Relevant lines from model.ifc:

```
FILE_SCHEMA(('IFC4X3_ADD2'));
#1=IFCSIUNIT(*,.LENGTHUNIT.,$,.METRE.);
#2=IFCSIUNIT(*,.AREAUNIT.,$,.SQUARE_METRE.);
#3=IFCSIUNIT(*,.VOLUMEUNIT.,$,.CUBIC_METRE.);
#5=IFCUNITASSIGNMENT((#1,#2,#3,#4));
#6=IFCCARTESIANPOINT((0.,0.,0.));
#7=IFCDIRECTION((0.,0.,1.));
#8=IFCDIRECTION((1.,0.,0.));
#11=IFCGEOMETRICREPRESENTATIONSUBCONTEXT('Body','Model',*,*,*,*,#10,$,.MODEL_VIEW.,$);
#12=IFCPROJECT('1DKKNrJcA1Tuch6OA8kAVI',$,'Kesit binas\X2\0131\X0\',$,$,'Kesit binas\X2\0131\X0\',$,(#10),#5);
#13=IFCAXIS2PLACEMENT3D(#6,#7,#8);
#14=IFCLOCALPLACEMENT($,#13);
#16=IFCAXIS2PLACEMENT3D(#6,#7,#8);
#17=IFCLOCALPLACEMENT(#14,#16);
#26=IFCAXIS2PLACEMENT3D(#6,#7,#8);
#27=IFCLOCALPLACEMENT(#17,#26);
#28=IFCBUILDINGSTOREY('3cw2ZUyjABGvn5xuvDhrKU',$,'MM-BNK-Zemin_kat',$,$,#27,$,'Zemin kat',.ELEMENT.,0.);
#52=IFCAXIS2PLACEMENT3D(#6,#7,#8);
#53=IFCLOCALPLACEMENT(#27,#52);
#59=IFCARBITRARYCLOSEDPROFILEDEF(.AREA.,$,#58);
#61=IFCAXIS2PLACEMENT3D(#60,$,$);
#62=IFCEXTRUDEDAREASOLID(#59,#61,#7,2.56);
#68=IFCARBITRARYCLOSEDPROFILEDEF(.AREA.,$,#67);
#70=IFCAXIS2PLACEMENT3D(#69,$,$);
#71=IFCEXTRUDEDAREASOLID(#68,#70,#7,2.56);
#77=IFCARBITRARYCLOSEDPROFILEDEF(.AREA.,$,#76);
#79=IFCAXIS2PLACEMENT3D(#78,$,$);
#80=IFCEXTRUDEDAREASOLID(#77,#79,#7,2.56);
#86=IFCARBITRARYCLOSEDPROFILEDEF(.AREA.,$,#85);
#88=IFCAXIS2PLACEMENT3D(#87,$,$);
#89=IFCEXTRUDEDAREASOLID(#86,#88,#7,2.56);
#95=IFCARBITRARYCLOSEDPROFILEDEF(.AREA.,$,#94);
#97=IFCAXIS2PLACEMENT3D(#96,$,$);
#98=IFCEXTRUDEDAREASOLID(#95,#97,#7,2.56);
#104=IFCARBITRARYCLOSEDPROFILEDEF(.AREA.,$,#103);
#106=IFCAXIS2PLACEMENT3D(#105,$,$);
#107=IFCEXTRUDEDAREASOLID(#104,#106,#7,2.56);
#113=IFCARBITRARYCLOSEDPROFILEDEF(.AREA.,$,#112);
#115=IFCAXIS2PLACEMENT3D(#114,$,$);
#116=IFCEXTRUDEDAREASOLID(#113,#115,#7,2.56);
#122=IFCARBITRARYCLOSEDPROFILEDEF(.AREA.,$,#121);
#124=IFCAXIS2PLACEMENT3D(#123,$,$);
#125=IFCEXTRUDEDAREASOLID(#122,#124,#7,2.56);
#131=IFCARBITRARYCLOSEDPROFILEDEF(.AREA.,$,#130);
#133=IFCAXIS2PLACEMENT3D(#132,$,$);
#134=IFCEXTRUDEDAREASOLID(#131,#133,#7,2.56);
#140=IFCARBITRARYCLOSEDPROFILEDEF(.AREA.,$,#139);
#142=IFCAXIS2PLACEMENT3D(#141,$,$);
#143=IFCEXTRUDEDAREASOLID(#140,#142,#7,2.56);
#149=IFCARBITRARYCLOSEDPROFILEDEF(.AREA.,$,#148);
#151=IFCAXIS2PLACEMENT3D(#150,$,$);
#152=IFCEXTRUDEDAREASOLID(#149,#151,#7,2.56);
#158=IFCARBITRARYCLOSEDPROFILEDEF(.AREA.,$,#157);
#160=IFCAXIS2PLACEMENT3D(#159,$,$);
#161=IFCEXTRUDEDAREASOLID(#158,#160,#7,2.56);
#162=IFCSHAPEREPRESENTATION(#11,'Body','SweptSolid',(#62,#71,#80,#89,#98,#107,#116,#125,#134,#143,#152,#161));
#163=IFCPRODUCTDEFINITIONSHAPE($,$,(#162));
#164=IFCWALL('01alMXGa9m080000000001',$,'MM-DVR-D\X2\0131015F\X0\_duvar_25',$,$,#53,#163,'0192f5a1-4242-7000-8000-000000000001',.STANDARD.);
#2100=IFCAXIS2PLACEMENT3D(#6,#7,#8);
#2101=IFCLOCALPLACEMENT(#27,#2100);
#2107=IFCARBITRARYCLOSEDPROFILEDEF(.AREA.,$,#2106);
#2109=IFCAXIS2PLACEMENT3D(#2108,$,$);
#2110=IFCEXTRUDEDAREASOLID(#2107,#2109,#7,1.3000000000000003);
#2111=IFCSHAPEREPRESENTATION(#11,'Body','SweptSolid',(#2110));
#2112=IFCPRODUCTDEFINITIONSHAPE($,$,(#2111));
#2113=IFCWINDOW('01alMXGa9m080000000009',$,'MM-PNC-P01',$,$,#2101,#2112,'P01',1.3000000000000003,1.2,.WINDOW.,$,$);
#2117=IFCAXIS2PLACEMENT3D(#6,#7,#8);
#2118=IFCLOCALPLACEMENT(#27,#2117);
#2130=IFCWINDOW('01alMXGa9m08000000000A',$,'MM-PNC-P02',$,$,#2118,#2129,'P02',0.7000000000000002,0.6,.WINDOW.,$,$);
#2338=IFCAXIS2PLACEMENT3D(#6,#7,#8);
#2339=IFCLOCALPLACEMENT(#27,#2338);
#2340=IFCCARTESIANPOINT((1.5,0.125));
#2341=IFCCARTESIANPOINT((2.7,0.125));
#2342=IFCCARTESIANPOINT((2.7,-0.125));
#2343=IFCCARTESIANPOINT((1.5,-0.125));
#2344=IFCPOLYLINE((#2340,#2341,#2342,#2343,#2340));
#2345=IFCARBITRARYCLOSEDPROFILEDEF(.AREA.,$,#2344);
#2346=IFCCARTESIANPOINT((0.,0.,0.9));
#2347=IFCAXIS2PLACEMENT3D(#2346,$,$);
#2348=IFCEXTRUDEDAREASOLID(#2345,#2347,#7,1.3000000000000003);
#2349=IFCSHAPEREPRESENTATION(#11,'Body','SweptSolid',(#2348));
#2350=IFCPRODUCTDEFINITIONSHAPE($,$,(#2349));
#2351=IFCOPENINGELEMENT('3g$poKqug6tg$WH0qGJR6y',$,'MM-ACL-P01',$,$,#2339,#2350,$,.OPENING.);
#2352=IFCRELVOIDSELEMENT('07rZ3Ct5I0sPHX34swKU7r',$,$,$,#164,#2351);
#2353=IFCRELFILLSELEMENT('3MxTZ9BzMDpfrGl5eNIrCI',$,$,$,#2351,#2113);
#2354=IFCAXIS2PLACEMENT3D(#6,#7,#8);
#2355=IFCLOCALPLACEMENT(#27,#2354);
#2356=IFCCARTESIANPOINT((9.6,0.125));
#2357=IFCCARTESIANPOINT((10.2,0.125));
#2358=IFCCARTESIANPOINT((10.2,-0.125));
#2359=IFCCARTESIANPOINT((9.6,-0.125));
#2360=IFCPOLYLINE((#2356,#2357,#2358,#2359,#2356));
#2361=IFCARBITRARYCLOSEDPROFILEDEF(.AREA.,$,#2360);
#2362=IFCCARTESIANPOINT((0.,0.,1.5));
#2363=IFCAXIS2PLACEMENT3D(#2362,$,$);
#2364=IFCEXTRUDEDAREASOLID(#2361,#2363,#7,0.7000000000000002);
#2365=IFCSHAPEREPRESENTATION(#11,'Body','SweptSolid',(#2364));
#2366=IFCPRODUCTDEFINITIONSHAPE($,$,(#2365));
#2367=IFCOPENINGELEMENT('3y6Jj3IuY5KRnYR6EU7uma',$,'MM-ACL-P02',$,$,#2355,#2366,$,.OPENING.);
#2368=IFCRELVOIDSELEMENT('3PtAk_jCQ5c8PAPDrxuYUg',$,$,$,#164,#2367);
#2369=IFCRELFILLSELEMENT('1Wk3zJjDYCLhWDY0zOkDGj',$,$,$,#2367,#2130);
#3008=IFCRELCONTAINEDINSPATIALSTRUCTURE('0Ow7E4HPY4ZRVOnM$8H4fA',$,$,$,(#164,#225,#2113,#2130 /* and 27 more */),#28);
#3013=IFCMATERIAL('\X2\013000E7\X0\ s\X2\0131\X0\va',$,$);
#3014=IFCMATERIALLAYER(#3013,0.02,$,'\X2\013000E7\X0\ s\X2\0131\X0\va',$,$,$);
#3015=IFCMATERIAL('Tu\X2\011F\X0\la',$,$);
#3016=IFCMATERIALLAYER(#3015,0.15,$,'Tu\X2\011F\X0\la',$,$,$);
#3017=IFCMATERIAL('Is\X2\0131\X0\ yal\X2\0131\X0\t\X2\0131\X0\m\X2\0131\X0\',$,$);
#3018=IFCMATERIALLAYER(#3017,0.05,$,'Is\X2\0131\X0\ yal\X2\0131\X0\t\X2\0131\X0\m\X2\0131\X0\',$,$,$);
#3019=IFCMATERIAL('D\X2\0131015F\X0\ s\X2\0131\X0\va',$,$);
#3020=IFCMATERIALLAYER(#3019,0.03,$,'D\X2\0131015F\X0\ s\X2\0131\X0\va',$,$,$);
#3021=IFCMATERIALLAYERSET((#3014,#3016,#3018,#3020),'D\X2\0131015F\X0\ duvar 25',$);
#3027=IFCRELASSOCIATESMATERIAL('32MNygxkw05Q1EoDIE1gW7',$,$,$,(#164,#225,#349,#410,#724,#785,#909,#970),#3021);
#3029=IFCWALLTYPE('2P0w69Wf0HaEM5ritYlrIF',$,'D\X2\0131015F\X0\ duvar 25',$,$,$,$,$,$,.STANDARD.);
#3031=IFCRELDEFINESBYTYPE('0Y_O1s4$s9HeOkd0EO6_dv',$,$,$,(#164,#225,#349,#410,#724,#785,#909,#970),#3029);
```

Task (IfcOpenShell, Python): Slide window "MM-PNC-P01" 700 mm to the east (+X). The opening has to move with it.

```python
import ifcopenshell
import ifcopenshell.api.geometry
import ifcopenshell.util.placement
import ifcopenshell.util.unit

model = ifcopenshell.open("model.ifc")
unit_scale = ifcopenshell.util.unit.calculate_unit_scale(model)

window = model.by_guid("01alMXGa9m080000000009")
opening = window.FillsVoids[0].RelatingOpeningElement
wall = opening.VoidsElements[0].RelatingBuildingElement

wall_matrix = ifcopenshell.util.placement.get_local_placement(wall.ObjectPlacement)
shift = wall_matrix[:3, 0] * 0.7 / unit_scale
before = ifcopenshell.util.placement.get_local_placement(window.ObjectPlacement)[:3, 3].copy()

# The window is not placed relative to its opening, so move both.
for product in (opening, window):
    matrix = ifcopenshell.util.placement.get_local_placement(product.ObjectPlacement)
    matrix[:3, 3] += shift
    ifcopenshell.api.geometry.edit_object_placement(model, product=product, matrix=matrix, is_si=False)

after = ifcopenshell.util.placement.get_local_placement(window.ObjectPlacement)[:3, 3]
print("window moved by", (after - before).round(3) + 0.0)

model.write("model_v2.ifc")
```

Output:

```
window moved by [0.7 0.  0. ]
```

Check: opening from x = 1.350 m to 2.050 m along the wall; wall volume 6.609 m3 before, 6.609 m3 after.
